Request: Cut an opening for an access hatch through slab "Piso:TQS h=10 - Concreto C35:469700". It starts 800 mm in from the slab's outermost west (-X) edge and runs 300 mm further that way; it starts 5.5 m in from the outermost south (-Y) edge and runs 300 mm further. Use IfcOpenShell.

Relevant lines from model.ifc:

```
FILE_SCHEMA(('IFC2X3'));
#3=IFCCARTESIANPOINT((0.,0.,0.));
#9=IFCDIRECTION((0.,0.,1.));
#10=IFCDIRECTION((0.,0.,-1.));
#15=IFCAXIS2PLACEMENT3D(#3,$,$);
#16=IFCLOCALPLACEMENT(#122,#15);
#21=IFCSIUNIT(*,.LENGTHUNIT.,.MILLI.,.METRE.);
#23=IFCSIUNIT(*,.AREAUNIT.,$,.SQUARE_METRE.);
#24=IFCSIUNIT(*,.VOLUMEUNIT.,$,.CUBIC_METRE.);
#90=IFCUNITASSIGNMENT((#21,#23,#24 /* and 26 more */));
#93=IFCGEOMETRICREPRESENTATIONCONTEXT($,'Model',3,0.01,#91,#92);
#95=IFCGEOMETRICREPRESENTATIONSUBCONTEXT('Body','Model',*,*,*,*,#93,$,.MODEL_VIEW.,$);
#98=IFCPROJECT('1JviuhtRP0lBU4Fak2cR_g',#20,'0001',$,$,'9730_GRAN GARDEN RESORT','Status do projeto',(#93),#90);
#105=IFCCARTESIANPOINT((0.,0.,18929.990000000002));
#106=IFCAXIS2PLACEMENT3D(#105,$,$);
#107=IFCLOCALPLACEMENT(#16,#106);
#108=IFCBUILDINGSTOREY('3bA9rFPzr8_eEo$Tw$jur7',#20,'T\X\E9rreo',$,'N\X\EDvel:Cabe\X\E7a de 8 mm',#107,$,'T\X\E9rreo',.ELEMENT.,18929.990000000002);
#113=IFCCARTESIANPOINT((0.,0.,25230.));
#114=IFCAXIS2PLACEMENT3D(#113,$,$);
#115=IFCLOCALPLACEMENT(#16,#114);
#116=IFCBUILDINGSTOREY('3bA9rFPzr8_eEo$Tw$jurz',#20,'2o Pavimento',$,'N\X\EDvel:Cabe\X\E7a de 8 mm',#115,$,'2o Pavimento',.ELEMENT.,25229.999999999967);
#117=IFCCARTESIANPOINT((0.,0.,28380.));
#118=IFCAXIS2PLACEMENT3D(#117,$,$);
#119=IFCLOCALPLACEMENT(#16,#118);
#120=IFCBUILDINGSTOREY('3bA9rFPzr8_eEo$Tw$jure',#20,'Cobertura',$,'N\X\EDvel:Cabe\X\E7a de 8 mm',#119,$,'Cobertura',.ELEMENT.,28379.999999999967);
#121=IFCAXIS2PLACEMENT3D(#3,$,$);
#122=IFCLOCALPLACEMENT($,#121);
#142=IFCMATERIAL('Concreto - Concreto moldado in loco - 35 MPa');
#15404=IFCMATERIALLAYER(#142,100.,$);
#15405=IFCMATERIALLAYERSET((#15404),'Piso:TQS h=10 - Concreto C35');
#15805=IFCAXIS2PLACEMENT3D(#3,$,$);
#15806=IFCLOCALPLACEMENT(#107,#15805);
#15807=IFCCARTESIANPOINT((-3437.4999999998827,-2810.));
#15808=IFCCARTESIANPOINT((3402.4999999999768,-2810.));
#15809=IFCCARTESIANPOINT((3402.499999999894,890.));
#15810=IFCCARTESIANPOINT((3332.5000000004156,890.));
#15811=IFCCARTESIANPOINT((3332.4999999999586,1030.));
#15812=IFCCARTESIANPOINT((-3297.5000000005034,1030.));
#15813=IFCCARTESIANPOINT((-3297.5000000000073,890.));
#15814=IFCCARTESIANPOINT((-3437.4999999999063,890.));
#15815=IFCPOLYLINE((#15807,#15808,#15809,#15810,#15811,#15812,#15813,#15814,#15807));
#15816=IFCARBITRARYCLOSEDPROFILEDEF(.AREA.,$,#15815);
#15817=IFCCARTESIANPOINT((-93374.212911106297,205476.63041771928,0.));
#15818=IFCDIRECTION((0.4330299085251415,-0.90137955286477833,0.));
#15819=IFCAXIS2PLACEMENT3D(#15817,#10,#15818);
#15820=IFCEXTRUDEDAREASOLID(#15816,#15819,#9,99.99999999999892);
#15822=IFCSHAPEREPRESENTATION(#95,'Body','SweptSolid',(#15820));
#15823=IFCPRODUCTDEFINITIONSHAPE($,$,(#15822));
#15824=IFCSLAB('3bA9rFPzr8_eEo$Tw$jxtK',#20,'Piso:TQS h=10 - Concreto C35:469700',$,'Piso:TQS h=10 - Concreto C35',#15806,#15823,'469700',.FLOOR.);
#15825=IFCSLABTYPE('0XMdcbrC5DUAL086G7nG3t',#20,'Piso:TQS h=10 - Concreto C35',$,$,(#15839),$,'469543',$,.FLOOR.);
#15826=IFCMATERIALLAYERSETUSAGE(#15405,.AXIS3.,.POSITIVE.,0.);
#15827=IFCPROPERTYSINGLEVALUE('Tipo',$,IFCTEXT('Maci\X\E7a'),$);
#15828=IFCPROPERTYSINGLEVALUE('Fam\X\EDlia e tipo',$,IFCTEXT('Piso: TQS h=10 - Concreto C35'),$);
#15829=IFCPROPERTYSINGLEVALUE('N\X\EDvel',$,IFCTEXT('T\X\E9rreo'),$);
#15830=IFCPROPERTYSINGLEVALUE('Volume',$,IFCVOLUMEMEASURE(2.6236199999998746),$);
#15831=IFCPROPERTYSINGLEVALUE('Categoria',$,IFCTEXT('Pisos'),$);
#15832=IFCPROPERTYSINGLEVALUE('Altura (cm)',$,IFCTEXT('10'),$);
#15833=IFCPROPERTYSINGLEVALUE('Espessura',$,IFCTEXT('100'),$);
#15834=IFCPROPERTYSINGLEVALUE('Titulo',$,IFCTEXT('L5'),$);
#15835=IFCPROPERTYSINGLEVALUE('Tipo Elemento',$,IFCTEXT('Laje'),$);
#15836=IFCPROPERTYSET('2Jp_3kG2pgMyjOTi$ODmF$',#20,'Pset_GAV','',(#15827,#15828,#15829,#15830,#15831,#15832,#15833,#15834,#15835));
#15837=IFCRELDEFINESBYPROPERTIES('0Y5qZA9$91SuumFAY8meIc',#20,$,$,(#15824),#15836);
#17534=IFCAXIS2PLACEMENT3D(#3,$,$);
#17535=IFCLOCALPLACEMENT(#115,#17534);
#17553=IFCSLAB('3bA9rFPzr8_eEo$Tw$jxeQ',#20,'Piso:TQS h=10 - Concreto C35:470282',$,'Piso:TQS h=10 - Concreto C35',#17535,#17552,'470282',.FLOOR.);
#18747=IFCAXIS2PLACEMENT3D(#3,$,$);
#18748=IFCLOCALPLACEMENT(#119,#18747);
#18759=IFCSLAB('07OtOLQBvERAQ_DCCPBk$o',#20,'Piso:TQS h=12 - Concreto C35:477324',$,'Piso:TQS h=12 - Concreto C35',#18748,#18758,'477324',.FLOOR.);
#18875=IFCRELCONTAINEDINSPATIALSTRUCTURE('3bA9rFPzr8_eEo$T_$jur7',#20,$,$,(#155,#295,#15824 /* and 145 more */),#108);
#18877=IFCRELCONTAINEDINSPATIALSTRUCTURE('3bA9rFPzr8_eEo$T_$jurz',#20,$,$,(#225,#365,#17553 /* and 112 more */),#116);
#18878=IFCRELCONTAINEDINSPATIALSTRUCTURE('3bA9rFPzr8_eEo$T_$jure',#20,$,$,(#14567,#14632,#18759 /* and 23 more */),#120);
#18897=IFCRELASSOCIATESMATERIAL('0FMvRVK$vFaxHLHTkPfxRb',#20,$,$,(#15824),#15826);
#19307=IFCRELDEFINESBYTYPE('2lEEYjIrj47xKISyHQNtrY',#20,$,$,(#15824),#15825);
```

```python
import numpy as np
import ifcopenshell
import ifcopenshell.api.feature
import ifcopenshell.api.geometry
import ifcopenshell.api.pset
import ifcopenshell.api.root
import ifcopenshell.geom
import ifcopenshell.util.element
import ifcopenshell.util.placement
import ifcopenshell.util.representation
import ifcopenshell.util.shape
import ifcopenshell.util.unit

model = ifcopenshell.open("model.ifc")
unit_scale = ifcopenshell.util.unit.calculate_unit_scale(model)
volume_scale = ifcopenshell.util.unit.calculate_unit_scale(model, "VOLUMEUNIT")
settings = ifcopenshell.geom.settings()


def volume(element):
    """Net volume in cubic metres, openings subtracted."""
    shape = ifcopenshell.geom.create_shape(settings, element)
    return ifcopenshell.util.shape.get_volume(shape.geometry)


slab = model.by_guid("3bA9rFPzr8_eEo$Tw$jxtK")
before = volume(slab)

# Extent in the slab's own axes, in metres. The edges named are its -X and -Y sides.
slab_shape = ifcopenshell.geom.create_shape(settings, slab)
vertices = ifcopenshell.util.shape.get_vertices(slab_shape.geometry)
x_min, y_min, bottom = vertices.min(axis=0)
top = vertices[:, 2].max()

opening = ifcopenshell.api.root.create_entity(model, ifc_class="IfcOpeningElement", name="Access hatch opening")
context = ifcopenshell.util.representation.get_context(model, "Model", "Body", "MODEL_VIEW")
width, depth = 0.3, 0.3
outline = [(0.0, 0.0), (width, 0.0), (width, depth), (0.0, depth), (0.0, 0.0)]
# Overshoot both faces by 50 mm so the cut is clean.
shape = ifcopenshell.api.geometry.add_slab_representation(
    model, context=context, depth=top - bottom + 0.1, polyline=outline
)
ifcopenshell.api.geometry.assign_representation(model, product=opening, representation=shape)

matrix = ifcopenshell.util.placement.get_local_placement(slab.ObjectPlacement)
matrix[:, 3] = matrix @ np.append(np.array([x_min + 0.8, y_min + 5.5, bottom - 0.05]) / unit_scale, 1.0)
ifcopenshell.api.geometry.edit_object_placement(model, product=opening, matrix=matrix, is_si=False)
ifcopenshell.api.feature.add_feature(model, feature=opening, element=slab)

after = volume(slab)

# Update the slab's stored quantities.
pset = model.by_id(ifcopenshell.util.element.get_pset(slab, "Pset_GAV", should_inherit=False)["id"])
ifcopenshell.api.pset.edit_pset(model, pset=pset, properties={
    "Volume": model.create_entity("IfcVolumeMeasure", after / volume_scale),
})

print(f"slab volume {before:.3f} -> {after:.3f} m3")

model.write("model_edited.ifc")
```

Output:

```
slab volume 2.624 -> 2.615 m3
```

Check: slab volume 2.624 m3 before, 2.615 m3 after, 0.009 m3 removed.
